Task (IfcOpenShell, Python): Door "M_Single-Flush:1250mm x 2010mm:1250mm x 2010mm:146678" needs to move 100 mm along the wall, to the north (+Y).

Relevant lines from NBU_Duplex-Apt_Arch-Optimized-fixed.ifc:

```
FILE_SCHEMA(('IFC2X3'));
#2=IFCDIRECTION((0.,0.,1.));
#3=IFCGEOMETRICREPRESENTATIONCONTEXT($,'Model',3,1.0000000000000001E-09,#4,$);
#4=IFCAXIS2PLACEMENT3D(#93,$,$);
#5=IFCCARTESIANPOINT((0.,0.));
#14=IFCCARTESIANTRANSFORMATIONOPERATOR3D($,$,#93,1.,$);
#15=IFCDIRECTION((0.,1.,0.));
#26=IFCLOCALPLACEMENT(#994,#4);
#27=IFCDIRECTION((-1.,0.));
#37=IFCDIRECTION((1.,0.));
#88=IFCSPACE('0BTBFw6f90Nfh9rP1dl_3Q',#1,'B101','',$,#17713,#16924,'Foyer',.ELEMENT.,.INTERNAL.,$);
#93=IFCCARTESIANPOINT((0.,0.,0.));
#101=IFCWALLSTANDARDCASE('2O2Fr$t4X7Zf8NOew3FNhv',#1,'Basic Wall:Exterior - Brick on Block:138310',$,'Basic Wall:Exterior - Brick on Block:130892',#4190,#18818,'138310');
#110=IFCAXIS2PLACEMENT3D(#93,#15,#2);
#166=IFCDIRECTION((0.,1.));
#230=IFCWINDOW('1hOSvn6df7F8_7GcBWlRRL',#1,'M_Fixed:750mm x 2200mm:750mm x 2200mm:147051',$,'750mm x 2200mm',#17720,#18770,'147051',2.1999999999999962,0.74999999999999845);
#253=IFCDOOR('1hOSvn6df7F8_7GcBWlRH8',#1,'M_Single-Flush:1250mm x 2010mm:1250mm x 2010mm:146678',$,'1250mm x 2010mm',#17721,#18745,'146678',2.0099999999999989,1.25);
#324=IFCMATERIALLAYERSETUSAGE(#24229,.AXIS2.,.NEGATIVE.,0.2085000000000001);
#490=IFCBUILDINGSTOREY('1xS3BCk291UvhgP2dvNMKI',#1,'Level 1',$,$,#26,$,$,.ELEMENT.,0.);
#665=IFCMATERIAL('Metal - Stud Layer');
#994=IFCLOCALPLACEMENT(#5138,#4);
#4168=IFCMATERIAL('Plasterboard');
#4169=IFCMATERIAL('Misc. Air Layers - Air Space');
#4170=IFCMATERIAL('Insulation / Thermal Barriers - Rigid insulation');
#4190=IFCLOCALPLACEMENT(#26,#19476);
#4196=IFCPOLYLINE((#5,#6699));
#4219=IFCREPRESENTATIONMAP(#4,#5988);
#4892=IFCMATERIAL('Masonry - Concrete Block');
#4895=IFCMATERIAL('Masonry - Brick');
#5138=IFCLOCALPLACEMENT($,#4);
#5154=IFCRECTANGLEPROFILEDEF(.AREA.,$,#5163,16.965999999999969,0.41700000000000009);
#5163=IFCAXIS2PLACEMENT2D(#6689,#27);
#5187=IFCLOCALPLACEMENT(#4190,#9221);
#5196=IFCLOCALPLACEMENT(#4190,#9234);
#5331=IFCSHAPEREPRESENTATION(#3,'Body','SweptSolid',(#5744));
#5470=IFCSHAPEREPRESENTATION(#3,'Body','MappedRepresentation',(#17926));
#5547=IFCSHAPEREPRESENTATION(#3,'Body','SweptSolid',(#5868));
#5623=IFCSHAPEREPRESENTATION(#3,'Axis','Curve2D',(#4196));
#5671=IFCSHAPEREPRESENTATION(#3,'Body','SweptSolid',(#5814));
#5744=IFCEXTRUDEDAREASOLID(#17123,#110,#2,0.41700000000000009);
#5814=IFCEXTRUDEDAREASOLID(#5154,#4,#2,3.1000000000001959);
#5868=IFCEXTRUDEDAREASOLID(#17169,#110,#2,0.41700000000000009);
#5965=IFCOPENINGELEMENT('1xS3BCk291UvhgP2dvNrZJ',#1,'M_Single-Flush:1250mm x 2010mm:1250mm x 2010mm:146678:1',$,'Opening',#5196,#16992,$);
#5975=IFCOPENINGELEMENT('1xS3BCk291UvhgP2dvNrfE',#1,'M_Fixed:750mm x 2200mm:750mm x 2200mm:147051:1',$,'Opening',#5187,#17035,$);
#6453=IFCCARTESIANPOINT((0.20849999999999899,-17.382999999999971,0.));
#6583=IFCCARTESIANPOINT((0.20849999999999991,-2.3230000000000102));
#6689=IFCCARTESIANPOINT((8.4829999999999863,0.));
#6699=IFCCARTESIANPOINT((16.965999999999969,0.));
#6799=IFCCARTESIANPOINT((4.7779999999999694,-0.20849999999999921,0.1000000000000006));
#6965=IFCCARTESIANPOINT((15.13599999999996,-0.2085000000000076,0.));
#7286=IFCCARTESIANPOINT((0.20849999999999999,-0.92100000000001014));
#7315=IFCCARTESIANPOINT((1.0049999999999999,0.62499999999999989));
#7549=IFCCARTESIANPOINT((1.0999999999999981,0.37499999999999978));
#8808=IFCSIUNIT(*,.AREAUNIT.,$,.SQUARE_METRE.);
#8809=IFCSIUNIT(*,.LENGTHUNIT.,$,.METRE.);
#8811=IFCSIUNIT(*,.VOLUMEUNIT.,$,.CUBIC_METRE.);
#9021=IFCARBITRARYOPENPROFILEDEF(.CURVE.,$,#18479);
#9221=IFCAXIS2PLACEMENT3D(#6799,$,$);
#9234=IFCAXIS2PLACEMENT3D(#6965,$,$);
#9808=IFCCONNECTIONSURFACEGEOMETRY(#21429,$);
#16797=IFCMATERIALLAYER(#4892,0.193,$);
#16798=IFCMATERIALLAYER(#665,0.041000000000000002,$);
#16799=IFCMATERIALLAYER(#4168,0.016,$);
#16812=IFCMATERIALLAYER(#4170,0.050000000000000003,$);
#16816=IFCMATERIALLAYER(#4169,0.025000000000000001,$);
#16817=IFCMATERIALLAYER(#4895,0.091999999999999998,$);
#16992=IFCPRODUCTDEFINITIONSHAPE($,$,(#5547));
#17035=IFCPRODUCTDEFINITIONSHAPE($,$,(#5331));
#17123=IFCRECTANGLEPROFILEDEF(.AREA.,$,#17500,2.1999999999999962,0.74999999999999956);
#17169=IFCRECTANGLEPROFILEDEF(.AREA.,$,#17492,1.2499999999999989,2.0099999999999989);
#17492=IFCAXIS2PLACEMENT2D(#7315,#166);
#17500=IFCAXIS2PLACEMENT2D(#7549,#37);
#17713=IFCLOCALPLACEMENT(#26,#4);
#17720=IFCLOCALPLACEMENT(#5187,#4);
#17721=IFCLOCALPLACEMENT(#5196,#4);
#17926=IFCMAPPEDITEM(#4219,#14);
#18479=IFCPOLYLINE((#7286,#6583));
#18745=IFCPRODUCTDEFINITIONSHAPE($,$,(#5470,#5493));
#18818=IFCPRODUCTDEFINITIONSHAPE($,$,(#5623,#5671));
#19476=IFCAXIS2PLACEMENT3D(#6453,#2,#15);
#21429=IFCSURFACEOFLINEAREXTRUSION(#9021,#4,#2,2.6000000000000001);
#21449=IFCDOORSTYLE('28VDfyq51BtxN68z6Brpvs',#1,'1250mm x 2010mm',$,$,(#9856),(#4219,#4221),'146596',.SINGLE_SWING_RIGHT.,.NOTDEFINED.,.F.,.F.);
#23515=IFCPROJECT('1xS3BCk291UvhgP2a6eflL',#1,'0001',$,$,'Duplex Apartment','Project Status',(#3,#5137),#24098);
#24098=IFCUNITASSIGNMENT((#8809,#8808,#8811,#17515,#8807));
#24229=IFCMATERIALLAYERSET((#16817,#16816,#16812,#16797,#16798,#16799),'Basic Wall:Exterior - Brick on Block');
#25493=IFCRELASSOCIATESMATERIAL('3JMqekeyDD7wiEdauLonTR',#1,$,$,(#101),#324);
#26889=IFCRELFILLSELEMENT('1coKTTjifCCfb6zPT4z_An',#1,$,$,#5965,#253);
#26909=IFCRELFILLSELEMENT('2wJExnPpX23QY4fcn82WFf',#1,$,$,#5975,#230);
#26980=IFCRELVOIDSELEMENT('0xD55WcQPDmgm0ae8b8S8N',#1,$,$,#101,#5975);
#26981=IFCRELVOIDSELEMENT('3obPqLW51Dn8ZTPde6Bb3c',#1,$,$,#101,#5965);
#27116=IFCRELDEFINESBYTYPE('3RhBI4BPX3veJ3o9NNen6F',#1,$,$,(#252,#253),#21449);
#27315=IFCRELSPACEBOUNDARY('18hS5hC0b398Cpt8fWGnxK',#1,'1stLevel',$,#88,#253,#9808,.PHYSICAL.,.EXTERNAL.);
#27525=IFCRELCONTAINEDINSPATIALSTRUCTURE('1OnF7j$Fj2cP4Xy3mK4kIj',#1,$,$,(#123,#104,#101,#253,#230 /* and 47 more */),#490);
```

```python
import numpy as np
import ifcopenshell
import ifcopenshell.api.geometry
import ifcopenshell.util.placement

model = ifcopenshell.open("NBU_Duplex-Apt_Arch-Optimized-fixed.ifc")

door = model.by_id(253)
opening = door.FillsVoids[0].RelatingOpeningElement
wall = opening.VoidsElements[0].RelatingBuildingElement

wall_matrix = ifcopenshell.util.placement.get_local_placement(wall.ObjectPlacement)
shift = wall_matrix[:3, 0] * 0.1
before = ifcopenshell.util.placement.get_local_placement(door.ObjectPlacement)[:3, 3].copy()

# The door is placed relative to its opening, so it follows when the opening moves.
matrix = ifcopenshell.util.placement.get_local_placement(opening.ObjectPlacement)
matrix[:3, 3] += shift
ifcopenshell.api.geometry.edit_object_placement(
    model, product=opening, matrix=matrix, is_si=False, should_transform_children=True
)

# Space boundary surfaces are stored in each space's coordinates; move them too.
for rel in door.ProvidesBoundaries:
    if not rel.ConnectionGeometry:
        continue
    surface = rel.ConnectionGeometry.SurfaceOnRelatingElement
    space_matrix = ifcopenshell.util.placement.get_local_placement(rel.RelatingSpace.ObjectPlacement)
    point = np.array(surface.Position.Location.Coordinates) + space_matrix[:3, :3].T @ shift
    surface.Position = model.createIfcAxis2Placement3D(
        model.createIfcCartesianPoint(point.tolist()), surface.Position.Axis, surface.Position.RefDirection
    )

after = ifcopenshell.util.placement.get_local_placement(door.ObjectPlacement)[:3, 3]
print("door moved by", (after - before).round(3) + 0.0)

model.write("NBU_Duplex-Apt_Arch-Optimized-fixed_updated.ifc")
```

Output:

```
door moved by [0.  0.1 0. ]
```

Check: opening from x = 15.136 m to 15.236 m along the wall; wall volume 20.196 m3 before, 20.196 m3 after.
